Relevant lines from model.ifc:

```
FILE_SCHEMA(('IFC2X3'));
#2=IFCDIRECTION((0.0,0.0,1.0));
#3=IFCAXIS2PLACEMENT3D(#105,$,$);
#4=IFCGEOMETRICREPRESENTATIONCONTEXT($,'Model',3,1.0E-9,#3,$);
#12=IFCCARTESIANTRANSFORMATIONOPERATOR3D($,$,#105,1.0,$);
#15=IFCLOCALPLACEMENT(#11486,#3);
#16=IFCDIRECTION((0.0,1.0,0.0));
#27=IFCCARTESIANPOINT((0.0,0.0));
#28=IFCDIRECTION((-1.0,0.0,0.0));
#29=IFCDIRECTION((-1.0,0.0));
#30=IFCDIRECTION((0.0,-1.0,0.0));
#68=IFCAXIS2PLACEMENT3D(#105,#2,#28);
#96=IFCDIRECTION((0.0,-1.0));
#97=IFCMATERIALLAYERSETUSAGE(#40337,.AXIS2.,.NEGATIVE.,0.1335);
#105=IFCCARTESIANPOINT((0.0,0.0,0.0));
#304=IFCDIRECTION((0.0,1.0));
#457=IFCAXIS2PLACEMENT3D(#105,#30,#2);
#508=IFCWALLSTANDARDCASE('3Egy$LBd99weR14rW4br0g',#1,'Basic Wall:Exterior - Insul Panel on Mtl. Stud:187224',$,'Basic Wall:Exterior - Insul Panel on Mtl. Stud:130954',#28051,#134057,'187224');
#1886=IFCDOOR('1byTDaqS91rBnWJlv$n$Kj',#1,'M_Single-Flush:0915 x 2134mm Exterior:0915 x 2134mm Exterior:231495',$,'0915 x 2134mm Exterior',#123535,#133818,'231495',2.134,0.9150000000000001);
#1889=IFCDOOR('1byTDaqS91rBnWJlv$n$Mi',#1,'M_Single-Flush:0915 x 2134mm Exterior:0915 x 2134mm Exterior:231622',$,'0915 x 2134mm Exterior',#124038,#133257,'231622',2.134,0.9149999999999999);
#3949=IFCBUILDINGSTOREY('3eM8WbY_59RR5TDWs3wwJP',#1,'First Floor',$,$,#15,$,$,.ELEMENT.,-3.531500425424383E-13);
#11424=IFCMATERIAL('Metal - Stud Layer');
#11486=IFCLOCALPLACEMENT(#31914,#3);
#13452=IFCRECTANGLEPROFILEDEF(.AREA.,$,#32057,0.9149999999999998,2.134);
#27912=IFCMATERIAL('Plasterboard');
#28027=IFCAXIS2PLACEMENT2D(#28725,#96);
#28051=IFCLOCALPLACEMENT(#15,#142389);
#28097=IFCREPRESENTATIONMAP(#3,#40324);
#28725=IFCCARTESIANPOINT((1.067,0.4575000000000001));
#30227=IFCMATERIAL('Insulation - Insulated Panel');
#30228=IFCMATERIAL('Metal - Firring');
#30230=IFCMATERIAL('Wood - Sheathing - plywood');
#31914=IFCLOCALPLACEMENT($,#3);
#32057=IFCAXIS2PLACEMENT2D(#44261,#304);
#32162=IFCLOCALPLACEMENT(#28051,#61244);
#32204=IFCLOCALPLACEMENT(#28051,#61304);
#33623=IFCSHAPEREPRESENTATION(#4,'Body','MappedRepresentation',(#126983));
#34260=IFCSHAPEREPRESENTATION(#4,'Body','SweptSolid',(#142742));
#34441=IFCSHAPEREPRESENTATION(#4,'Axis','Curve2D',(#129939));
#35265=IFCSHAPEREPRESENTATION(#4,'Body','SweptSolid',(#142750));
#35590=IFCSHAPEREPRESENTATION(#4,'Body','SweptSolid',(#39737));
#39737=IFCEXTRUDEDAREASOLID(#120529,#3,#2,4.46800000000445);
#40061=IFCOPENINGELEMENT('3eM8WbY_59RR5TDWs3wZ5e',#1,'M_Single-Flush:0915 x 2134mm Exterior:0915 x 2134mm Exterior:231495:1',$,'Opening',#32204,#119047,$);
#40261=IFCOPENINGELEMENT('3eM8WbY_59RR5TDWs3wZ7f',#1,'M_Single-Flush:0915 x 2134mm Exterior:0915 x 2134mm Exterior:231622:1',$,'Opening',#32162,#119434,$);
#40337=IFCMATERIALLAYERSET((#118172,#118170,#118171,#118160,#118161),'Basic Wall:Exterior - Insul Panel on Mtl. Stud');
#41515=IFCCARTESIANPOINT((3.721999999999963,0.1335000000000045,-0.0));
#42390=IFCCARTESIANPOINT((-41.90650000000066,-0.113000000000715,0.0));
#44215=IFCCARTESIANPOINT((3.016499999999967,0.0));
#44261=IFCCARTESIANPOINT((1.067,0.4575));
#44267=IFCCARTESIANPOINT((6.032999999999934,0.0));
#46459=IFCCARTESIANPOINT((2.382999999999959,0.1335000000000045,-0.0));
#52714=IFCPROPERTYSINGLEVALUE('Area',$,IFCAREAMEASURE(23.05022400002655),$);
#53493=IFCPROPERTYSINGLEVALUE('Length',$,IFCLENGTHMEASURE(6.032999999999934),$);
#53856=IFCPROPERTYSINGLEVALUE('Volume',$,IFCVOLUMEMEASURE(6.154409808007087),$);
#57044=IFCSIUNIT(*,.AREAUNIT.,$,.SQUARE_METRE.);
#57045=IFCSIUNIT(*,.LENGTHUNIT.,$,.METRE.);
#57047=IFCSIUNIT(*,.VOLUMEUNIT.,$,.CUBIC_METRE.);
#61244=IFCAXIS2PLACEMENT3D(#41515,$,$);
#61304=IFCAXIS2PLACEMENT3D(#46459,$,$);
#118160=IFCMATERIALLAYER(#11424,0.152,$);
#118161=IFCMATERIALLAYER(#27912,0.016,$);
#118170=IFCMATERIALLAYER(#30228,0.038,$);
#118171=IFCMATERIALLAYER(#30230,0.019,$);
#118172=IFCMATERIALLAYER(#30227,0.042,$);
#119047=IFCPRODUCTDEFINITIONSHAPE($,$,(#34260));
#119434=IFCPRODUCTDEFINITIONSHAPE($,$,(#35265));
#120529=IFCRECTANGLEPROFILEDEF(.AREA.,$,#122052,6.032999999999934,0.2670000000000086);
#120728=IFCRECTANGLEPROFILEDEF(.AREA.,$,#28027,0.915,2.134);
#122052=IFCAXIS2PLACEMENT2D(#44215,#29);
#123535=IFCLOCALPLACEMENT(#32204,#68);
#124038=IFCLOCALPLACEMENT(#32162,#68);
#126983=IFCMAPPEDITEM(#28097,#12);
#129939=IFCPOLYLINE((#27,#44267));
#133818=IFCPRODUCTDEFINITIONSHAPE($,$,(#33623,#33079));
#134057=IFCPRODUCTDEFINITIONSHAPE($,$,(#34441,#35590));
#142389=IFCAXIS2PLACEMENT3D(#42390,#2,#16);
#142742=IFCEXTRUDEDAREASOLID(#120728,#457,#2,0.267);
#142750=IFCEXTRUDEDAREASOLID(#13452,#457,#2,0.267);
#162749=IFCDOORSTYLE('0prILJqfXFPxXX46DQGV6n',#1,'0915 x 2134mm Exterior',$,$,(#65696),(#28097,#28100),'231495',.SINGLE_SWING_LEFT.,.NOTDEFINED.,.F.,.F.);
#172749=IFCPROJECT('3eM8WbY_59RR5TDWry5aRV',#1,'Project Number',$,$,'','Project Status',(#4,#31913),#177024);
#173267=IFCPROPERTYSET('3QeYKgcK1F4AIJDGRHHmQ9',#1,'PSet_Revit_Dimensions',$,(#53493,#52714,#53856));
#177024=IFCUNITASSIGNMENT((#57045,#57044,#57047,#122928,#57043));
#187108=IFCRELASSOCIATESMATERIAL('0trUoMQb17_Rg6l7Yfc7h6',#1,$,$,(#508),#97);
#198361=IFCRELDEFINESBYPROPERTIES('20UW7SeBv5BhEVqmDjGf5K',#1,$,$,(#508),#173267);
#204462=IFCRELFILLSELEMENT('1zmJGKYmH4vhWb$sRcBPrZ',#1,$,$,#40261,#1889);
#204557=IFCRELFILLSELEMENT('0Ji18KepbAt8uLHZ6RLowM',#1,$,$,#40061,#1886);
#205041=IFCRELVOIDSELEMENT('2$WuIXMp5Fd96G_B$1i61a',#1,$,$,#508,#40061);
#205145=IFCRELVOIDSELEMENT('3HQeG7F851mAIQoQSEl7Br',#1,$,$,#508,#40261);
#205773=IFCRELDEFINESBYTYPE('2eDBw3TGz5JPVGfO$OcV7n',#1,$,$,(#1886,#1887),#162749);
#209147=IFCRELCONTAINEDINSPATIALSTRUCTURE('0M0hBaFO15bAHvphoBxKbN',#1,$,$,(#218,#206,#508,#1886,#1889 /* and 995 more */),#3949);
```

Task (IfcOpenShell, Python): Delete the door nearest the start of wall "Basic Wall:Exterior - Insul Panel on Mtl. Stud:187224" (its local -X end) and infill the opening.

```python
import ifcopenshell
import ifcopenshell.api.feature
import ifcopenshell.api.pset
import ifcopenshell.api.root
import ifcopenshell.geom
import ifcopenshell.util.element
import ifcopenshell.util.shape
import ifcopenshell.util.unit

model = ifcopenshell.open("model.ifc")
area_scale = ifcopenshell.util.unit.calculate_unit_scale(model, "AREAUNIT")
volume_scale = ifcopenshell.util.unit.calculate_unit_scale(model, "VOLUMEUNIT")
settings = ifcopenshell.geom.settings()


def volume(element):
    """Net volume in cubic metres, openings subtracted."""
    shape = ifcopenshell.geom.create_shape(settings, element)
    return ifcopenshell.util.shape.get_volume(shape.geometry)


door = model.by_guid("1byTDaqS91rBnWJlv$n$Kj")
opening = door.FillsVoids[0].RelatingOpeningElement
wall = opening.VoidsElements[0].RelatingBuildingElement
before = volume(wall)

ifcopenshell.api.root.remove_product(model, product=door)
ifcopenshell.api.feature.remove_feature(model, feature=opening)

after = volume(wall)
thickness = 0.267  # wall thickness in metres

# Update the wall's stored quantities.
pset = model.by_id(ifcopenshell.util.element.get_pset(wall, "PSet_Revit_Dimensions", should_inherit=False)["id"])
ifcopenshell.api.pset.edit_pset(model, pset=pset, properties={
    "Area": model.create_entity("IfcAreaMeasure", after / thickness / area_scale),
    "Volume": model.create_entity("IfcVolumeMeasure", after / volume_scale),
})

print(f"wall volume {before:.3f} -> {after:.3f} m3")

model.write("model-out.ifc")
```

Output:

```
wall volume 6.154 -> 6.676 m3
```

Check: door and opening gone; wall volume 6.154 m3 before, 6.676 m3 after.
